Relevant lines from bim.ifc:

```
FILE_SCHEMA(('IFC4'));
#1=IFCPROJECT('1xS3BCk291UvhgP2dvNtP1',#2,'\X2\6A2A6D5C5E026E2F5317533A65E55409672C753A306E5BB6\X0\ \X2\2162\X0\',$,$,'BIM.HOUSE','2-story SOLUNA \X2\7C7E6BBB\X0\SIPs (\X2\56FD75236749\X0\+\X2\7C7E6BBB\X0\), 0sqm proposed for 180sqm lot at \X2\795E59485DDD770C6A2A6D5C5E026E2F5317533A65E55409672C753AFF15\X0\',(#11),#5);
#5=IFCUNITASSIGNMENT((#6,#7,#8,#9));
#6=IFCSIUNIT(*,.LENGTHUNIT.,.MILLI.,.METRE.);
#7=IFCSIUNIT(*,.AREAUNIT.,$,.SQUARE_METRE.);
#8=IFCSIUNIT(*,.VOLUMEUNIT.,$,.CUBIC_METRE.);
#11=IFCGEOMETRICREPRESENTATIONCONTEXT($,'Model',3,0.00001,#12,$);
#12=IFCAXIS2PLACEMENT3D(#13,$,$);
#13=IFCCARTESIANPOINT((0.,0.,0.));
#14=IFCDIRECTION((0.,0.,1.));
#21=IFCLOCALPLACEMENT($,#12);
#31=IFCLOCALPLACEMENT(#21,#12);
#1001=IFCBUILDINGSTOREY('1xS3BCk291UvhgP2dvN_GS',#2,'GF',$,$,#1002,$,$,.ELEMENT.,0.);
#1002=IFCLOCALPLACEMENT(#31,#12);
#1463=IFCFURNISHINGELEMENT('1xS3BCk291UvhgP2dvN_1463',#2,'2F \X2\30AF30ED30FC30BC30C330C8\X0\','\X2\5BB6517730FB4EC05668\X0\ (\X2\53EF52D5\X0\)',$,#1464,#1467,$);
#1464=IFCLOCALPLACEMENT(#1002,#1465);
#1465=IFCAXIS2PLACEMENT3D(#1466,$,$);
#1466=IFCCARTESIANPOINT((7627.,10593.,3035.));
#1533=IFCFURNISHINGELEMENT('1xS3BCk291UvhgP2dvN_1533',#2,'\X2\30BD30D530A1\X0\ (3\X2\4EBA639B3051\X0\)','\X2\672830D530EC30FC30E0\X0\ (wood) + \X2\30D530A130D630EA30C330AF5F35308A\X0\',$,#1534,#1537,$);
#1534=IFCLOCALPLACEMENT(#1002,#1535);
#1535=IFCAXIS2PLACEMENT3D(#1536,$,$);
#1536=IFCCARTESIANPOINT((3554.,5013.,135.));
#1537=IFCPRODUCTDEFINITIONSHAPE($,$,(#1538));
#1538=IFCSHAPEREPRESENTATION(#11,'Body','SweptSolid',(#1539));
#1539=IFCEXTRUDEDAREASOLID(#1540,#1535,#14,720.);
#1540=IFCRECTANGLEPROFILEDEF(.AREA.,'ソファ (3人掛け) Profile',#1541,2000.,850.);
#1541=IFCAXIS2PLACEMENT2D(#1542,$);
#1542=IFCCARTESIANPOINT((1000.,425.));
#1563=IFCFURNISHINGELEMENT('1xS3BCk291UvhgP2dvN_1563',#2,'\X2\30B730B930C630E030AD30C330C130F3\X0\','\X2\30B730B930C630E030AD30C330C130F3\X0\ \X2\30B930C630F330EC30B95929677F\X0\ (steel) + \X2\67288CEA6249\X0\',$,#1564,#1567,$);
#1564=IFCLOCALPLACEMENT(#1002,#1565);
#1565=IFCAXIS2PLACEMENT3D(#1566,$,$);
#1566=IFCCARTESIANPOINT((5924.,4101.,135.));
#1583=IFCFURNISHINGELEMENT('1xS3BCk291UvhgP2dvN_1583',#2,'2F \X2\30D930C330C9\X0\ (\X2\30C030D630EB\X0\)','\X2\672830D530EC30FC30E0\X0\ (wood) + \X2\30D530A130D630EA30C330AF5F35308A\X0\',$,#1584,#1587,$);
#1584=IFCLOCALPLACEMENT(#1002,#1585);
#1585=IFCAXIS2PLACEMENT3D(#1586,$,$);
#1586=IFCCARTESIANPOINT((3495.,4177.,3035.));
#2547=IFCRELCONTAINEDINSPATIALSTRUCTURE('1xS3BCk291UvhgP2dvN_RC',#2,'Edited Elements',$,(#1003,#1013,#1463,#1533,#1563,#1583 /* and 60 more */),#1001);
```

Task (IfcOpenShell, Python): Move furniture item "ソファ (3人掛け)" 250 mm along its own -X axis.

```python
import ifcopenshell
import ifcopenshell.api.geometry
import ifcopenshell.util.placement

model = ifcopenshell.open("bim.ifc")

item = model.by_guid("1xS3BCk291UvhgP2dvN_1533")
matrix = ifcopenshell.util.placement.get_local_placement(item.ObjectPlacement)
matrix[:3, 3] -= matrix[:3, 0] * 250.0
ifcopenshell.api.geometry.edit_object_placement(model, product=item, matrix=matrix, is_si=False)

print(ifcopenshell.util.placement.get_local_placement(item.ObjectPlacement).round(3) + 0.0)

model.write("bim-out.ifc")
```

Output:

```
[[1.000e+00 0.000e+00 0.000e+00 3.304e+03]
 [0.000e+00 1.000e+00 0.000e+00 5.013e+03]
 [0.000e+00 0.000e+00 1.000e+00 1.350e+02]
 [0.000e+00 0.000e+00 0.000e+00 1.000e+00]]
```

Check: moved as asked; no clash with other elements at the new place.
